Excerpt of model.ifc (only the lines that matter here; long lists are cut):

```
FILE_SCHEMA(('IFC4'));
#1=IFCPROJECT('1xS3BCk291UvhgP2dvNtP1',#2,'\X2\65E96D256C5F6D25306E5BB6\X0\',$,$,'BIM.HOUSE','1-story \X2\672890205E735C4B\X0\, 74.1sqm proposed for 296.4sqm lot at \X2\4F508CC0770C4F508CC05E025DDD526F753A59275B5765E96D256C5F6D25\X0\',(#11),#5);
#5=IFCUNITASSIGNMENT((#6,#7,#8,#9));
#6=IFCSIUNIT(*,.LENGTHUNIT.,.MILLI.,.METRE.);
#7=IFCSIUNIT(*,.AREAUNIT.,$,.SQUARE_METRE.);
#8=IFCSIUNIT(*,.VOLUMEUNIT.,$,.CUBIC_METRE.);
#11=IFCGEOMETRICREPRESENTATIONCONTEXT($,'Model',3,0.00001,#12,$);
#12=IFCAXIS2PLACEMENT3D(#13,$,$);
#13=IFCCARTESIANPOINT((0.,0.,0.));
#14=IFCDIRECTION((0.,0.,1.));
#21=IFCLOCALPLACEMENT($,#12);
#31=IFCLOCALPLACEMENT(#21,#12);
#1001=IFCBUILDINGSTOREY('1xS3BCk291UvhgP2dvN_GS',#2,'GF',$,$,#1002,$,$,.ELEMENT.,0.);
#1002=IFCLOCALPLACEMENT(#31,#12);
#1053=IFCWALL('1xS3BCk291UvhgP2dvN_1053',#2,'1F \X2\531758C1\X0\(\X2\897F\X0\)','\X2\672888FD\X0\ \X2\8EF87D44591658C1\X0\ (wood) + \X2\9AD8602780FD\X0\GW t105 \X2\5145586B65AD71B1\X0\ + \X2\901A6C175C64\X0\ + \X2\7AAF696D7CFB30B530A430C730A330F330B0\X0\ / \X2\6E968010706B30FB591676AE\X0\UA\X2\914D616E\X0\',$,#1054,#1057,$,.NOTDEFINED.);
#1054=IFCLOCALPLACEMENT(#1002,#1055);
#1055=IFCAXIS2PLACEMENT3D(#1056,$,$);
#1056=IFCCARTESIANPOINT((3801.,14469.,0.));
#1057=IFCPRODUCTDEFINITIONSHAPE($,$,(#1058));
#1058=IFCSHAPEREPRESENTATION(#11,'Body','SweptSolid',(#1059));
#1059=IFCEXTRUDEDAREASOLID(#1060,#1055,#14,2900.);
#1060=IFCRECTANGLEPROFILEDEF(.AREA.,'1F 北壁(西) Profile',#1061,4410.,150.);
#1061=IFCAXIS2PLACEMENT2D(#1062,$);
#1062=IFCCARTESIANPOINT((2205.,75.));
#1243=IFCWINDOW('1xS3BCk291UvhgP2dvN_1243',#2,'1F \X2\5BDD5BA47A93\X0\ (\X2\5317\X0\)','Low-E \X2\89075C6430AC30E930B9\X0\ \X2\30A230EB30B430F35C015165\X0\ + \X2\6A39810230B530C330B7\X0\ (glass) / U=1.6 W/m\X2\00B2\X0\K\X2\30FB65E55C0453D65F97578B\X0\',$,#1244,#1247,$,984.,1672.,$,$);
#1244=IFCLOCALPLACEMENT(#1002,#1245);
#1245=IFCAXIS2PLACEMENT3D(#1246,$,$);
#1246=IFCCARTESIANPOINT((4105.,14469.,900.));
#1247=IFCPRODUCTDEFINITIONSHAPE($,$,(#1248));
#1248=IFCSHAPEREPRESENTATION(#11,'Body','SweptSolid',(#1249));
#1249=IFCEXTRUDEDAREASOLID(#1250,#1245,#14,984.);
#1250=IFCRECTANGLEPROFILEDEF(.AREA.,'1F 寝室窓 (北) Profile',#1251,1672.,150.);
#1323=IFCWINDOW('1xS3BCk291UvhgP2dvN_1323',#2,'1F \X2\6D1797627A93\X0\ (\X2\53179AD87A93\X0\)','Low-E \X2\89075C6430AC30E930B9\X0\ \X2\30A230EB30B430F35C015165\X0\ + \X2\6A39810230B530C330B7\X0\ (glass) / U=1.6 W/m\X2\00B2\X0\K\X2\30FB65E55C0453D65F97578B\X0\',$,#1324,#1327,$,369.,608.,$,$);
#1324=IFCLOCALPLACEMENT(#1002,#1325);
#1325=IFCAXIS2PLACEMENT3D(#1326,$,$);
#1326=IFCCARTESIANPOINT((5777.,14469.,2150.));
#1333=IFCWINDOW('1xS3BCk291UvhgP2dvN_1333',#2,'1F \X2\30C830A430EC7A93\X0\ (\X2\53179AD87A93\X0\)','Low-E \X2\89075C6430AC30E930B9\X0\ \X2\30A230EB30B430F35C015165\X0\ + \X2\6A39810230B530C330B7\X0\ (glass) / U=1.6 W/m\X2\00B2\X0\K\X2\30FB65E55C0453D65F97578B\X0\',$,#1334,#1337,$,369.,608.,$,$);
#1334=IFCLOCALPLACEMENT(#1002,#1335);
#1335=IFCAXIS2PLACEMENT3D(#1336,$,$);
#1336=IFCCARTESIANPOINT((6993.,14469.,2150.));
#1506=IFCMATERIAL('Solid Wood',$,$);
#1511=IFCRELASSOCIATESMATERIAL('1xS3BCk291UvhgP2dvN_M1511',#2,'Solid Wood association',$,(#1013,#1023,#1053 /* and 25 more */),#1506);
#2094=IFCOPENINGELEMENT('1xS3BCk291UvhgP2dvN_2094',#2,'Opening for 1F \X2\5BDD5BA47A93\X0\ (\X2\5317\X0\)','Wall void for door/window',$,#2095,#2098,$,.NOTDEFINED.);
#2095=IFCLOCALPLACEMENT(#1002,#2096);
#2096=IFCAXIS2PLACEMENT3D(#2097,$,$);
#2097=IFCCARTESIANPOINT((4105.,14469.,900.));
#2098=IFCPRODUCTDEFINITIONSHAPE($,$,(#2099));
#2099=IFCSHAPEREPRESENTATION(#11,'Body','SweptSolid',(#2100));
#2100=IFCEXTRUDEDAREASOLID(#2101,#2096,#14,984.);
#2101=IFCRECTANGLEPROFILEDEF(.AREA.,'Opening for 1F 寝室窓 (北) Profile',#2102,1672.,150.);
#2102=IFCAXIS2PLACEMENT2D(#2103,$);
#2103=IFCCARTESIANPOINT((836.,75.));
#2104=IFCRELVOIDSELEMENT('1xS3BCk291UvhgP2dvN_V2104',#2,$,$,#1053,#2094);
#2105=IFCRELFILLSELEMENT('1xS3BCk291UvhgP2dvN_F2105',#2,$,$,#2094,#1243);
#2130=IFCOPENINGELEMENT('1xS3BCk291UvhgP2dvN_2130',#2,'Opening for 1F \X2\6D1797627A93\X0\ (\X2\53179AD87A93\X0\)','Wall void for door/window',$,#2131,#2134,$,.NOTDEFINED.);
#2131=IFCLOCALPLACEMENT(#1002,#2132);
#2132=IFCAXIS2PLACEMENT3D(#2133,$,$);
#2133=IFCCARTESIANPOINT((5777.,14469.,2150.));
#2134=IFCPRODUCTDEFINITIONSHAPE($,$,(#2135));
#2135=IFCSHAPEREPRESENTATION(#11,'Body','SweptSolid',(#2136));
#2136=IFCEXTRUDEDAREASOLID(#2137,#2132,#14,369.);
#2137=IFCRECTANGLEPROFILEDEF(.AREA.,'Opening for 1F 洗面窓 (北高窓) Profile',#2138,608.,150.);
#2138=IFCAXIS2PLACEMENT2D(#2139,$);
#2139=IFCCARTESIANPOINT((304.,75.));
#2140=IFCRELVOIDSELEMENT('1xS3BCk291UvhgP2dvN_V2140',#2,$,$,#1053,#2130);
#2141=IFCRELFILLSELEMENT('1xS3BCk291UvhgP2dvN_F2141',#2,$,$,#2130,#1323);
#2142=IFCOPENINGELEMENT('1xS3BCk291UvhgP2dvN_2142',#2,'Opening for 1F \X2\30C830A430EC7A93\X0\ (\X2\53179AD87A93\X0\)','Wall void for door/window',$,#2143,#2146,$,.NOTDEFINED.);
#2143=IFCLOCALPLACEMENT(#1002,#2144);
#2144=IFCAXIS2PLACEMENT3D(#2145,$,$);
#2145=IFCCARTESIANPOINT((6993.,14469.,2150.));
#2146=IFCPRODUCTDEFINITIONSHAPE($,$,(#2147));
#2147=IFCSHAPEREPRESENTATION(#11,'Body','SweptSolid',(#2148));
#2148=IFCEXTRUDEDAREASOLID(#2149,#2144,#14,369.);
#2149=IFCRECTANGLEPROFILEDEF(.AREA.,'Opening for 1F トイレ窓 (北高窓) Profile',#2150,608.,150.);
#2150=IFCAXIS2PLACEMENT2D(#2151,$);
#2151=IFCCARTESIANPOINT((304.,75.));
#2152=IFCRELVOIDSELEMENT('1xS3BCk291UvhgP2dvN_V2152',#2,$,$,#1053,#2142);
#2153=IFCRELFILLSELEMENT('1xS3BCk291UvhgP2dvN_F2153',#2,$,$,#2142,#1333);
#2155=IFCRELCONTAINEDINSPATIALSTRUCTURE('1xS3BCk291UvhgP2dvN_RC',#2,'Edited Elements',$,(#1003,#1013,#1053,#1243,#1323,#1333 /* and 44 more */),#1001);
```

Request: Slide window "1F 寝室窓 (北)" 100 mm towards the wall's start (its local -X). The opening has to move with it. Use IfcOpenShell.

```python
import ifcopenshell
import ifcopenshell.api.geometry
import ifcopenshell.util.placement

model = ifcopenshell.open("model.ifc")

window = model.by_guid("1xS3BCk291UvhgP2dvN_1243")
opening = window.FillsVoids[0].RelatingOpeningElement
wall = opening.VoidsElements[0].RelatingBuildingElement

wall_matrix = ifcopenshell.util.placement.get_local_placement(wall.ObjectPlacement)
shift = wall_matrix[:3, 0] * -100.0
before = ifcopenshell.util.placement.get_local_placement(window.ObjectPlacement)[:3, 3].copy()

# The window is not placed relative to its opening, so move both.
for product in (opening, window):
    matrix = ifcopenshell.util.placement.get_local_placement(product.ObjectPlacement)
    matrix[:3, 3] += shift
    ifcopenshell.api.geometry.edit_object_placement(model, product=product, matrix=matrix, is_si=False)

after = ifcopenshell.util.placement.get_local_placement(window.ObjectPlacement)[:3, 3]
print("window moved by", (after - before).round(3) + 0.0)

model.write("model_updated.ifc")
```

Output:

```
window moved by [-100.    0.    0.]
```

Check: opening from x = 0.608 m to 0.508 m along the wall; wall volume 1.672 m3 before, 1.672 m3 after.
